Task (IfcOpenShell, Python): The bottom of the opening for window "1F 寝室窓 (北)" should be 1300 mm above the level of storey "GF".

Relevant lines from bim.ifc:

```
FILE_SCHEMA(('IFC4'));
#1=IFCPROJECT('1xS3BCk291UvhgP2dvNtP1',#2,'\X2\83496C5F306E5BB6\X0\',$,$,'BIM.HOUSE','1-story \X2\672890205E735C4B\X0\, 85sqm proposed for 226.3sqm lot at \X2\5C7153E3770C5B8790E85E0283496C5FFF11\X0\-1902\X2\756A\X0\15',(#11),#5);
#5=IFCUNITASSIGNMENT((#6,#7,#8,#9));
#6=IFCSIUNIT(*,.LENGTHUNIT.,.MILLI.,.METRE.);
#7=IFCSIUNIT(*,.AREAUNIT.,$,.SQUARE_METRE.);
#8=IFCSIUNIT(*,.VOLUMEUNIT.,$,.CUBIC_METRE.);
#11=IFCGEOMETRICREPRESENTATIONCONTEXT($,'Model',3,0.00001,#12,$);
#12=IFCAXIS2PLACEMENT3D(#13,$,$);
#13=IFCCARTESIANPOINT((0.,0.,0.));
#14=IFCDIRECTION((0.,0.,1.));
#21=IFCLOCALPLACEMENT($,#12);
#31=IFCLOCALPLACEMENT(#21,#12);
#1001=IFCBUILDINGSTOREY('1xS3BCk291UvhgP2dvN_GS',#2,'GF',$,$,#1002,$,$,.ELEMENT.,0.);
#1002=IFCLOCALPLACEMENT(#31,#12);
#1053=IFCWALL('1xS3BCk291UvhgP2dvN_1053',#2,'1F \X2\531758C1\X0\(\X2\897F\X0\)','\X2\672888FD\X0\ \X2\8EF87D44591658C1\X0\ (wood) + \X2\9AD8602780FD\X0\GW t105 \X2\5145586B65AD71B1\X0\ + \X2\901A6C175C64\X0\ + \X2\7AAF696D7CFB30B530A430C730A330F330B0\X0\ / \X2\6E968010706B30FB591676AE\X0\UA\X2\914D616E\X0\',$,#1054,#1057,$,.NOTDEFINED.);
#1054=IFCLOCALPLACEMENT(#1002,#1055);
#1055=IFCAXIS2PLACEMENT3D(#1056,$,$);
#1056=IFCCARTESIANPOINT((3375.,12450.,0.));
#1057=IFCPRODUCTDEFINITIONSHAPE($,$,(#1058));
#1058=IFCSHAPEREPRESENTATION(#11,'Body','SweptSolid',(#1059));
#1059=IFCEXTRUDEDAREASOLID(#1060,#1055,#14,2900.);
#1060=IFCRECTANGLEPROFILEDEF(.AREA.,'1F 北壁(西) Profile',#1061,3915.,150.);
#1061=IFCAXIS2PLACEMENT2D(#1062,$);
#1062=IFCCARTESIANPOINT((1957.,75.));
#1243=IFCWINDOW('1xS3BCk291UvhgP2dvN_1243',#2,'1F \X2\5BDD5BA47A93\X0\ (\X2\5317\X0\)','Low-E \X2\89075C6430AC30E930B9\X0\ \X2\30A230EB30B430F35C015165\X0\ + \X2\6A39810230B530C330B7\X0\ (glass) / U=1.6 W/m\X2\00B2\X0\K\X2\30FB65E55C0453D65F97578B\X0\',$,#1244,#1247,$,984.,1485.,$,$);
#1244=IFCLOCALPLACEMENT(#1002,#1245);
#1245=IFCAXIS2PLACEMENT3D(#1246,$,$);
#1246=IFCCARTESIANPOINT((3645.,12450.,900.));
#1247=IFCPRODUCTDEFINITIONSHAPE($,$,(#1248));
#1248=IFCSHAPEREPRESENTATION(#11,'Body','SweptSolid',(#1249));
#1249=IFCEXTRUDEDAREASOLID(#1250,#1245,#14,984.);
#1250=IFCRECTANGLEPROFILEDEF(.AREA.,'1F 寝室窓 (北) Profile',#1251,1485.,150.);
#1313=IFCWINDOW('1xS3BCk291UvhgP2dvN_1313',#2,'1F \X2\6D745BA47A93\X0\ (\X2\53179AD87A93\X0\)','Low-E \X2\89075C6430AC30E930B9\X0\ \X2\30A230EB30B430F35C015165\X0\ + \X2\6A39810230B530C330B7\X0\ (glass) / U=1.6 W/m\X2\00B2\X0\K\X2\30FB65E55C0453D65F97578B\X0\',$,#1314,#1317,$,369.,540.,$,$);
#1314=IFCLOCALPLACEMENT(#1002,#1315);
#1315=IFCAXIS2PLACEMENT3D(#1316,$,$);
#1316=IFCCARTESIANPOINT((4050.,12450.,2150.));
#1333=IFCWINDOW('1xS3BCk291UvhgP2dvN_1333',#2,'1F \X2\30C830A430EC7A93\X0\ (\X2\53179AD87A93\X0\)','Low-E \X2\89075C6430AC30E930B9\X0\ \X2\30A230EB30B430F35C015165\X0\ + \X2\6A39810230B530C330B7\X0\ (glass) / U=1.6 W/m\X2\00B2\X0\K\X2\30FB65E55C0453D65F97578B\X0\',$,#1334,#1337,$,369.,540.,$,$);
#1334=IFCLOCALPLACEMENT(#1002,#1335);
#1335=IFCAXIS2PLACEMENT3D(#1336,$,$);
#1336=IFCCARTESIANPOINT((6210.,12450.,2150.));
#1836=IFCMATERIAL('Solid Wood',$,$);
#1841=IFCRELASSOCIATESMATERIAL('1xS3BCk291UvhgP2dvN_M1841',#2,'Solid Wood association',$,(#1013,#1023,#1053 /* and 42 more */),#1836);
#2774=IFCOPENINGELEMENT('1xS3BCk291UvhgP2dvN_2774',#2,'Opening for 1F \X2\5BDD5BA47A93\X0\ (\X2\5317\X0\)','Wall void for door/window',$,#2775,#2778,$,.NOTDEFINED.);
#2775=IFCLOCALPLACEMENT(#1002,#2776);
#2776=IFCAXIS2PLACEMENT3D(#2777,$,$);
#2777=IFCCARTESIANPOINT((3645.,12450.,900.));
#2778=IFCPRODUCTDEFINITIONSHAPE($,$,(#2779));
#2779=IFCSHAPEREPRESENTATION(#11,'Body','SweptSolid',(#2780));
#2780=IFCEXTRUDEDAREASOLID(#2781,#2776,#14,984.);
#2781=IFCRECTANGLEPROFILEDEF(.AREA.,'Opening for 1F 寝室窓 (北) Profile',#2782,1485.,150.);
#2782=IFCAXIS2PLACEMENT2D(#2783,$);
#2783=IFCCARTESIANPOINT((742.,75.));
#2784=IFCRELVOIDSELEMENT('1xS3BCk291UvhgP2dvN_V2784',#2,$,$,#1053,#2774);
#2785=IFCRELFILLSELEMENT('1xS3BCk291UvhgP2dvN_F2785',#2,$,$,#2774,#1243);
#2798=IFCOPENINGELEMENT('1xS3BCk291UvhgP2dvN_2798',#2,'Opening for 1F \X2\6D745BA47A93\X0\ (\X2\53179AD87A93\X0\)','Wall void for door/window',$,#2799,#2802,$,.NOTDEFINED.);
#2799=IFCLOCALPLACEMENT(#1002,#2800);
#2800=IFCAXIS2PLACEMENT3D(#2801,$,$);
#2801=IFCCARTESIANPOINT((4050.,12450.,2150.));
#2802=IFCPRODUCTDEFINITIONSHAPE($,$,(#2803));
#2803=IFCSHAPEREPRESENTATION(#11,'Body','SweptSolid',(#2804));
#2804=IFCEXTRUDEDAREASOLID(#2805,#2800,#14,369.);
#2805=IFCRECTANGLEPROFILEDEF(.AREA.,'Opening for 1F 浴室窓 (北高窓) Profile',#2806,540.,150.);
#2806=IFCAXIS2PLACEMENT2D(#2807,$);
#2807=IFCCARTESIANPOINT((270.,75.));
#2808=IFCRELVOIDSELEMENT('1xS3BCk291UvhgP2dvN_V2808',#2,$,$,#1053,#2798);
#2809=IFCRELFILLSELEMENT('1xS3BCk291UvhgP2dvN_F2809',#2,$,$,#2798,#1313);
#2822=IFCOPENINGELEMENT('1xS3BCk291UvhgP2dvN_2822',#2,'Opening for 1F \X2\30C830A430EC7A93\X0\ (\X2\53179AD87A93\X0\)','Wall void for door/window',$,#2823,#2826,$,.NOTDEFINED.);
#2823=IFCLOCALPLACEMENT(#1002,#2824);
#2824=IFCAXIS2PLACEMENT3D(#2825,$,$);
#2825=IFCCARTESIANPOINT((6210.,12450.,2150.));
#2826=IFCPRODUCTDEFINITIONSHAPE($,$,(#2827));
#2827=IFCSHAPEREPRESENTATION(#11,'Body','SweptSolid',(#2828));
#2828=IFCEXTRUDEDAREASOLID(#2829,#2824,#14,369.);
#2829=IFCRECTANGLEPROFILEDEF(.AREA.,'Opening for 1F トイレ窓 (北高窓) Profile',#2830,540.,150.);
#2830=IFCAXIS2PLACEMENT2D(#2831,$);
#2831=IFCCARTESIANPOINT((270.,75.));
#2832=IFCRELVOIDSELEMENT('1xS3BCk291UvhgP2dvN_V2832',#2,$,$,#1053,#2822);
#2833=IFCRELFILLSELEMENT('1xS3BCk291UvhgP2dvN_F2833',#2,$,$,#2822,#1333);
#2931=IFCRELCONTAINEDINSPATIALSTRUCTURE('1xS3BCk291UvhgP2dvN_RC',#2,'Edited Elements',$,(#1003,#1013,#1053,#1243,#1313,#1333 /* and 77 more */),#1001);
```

```python
import numpy as np
import ifcopenshell
import ifcopenshell.api.geometry
import ifcopenshell.geom
import ifcopenshell.util.element
import ifcopenshell.util.placement
import ifcopenshell.util.shape
import ifcopenshell.util.unit

model = ifcopenshell.open("bim.ifc")
unit_scale = ifcopenshell.util.unit.calculate_unit_scale(model)

window = model.by_id(1243)
opening = window.FillsVoids[0].RelatingOpeningElement
storey = ifcopenshell.util.element.get_container(window, ifc_class="IfcBuildingStorey")
level = ifcopenshell.util.placement.get_local_placement(storey.ObjectPlacement)[2, 3]

# The opening's origin need not be at the sill, so measure its lowest point.
shape = ifcopenshell.geom.create_shape(ifcopenshell.geom.settings(), opening)
bottom = ifcopenshell.util.shape.get_shape_bottom_elevation(shape, shape.geometry) / unit_scale
dz = level + 1.3 / unit_scale - bottom

shift = np.array([0.0, 0.0, dz])
# The window is not placed relative to its opening, so move both.
for product in (opening, window):
    matrix = ifcopenshell.util.placement.get_local_placement(product.ObjectPlacement)
    matrix[:3, 3] += shift
    ifcopenshell.api.geometry.edit_object_placement(model, product=product, matrix=matrix, is_si=False)

print(f"moved by {dz * unit_scale:+.3f} m")

model.write("bim_edited.ifc")
```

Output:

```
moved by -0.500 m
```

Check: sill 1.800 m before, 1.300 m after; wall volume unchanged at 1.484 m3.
